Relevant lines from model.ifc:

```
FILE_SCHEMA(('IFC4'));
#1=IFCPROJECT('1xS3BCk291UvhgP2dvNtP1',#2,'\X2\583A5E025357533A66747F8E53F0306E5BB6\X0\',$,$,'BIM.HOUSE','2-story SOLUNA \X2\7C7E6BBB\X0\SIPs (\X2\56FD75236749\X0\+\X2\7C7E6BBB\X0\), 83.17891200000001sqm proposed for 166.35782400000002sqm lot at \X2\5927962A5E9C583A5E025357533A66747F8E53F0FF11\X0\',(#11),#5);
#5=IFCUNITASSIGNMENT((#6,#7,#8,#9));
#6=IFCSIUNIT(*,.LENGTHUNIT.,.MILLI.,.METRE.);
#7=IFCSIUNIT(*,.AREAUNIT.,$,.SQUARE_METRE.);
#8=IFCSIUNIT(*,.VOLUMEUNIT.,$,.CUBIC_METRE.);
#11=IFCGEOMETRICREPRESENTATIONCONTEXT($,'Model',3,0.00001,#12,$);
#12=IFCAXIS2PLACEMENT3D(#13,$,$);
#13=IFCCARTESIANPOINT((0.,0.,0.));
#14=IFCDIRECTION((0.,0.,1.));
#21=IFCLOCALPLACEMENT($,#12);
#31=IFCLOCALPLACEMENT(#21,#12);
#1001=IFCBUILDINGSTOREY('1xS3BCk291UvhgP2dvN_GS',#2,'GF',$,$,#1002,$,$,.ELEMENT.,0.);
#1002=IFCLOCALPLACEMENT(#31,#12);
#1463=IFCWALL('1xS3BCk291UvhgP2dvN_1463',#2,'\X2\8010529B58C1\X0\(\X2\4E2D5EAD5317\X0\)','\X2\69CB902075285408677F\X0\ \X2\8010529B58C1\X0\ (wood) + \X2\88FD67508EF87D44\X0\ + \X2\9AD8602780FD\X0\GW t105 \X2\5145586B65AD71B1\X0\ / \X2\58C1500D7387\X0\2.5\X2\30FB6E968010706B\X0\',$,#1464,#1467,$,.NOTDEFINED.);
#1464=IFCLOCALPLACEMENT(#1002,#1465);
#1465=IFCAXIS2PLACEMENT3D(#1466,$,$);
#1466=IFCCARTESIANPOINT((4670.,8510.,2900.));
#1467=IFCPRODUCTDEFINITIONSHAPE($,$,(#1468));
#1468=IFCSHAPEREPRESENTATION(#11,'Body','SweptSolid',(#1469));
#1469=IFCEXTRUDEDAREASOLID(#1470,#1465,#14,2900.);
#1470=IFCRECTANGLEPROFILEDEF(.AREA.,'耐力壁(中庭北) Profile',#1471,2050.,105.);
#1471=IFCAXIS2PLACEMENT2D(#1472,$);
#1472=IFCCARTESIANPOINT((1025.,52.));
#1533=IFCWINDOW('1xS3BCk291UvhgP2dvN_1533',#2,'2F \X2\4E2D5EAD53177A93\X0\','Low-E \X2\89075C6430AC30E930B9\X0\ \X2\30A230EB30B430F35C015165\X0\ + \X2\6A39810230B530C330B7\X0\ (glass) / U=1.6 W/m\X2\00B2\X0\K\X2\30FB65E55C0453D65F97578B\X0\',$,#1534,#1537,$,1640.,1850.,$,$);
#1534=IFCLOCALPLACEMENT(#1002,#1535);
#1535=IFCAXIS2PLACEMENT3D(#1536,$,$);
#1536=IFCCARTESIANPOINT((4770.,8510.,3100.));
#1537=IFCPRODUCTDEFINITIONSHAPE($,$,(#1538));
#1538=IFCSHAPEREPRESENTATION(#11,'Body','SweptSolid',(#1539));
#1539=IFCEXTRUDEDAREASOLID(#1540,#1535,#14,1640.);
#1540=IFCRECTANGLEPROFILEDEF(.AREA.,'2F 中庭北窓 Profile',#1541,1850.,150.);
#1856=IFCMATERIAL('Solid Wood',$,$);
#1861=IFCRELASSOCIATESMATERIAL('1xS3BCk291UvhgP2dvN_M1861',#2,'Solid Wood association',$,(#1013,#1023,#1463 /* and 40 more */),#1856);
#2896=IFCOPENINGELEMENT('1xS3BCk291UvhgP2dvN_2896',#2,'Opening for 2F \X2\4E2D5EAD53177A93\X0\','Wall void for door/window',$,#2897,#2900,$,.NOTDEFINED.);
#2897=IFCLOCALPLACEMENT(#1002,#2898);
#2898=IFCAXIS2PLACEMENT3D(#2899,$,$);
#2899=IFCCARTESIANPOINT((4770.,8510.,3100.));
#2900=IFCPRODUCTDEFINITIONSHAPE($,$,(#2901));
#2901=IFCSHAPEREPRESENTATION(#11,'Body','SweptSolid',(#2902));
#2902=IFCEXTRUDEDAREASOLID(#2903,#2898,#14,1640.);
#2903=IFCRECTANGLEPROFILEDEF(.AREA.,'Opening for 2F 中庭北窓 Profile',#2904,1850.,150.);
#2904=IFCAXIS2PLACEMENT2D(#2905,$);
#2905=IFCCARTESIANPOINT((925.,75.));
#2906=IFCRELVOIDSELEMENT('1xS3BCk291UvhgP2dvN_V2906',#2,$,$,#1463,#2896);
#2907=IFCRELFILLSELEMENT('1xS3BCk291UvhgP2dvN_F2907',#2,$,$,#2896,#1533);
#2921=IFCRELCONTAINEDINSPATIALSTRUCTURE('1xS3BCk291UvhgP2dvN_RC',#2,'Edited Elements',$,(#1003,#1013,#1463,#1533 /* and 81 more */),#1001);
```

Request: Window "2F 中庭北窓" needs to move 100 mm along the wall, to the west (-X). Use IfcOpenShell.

```python
import ifcopenshell
import ifcopenshell.api.geometry
import ifcopenshell.util.placement

model = ifcopenshell.open("model.ifc")

window = model.by_id(1533)
opening = window.FillsVoids[0].RelatingOpeningElement
wall = opening.VoidsElements[0].RelatingBuildingElement

wall_matrix = ifcopenshell.util.placement.get_local_placement(wall.ObjectPlacement)
shift = wall_matrix[:3, 0] * -100.0
before = ifcopenshell.util.placement.get_local_placement(window.ObjectPlacement)[:3, 3].copy()

# The window is not placed relative to its opening, so move both.
for product in (opening, window):
    matrix = ifcopenshell.util.placement.get_local_placement(product.ObjectPlacement)
    matrix[:3, 3] += shift
    ifcopenshell.api.geometry.edit_object_placement(model, product=product, matrix=matrix, is_si=False)

after = ifcopenshell.util.placement.get_local_placement(window.ObjectPlacement)[:3, 3]
print("window moved by", (after - before).round(3) + 0.0)

model.write("model_v2.ifc")
```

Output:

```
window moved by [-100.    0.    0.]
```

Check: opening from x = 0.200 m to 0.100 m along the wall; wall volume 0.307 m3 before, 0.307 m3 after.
